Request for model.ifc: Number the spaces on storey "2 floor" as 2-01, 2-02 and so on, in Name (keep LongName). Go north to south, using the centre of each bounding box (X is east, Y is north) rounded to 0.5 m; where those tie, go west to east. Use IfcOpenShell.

First a look at what the model holds.

```python
import ifcopenshell
import ifcopenshell.util.element
import ifcopenshell.util.placement

model = ifcopenshell.open("model.ifc")
print(model.schema)
storey = next(s for s in model.by_type("IfcBuildingStorey") if s.Name == "2 floor")
spaces = [e for e in ifcopenshell.util.element.get_decomposition(storey) if e.is_a("IfcSpace")]
for e in sorted(spaces, key=lambda e: e.id()):
    origin = ifcopenshell.util.placement.get_local_placement(e.ObjectPlacement)[:3, 3]
    print(e.id(), e.Name, e.LongName, origin.round(2) + 0.0, sep=" | ")
```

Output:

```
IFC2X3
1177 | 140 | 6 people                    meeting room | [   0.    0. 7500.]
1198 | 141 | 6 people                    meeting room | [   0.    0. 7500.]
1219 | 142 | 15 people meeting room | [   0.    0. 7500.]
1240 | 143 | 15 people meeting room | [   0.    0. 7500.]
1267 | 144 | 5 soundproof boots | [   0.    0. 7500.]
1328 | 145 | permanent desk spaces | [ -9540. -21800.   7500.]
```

```python
import ifcopenshell
import ifcopenshell.geom
import ifcopenshell.util.element
import ifcopenshell.util.shape

model = ifcopenshell.open("model.ifc")
settings = ifcopenshell.geom.settings()
settings.set("use-world-coords", True)


def centre(element):
    shape = ifcopenshell.geom.create_shape(settings, element)
    return ifcopenshell.util.shape.get_bbox_centroid(shape.geometry)


storey = next(s for s in model.by_type("IfcBuildingStorey") if s.Name == "2 floor")
spaces = [e for e in ifcopenshell.util.element.get_decomposition(storey) if e.is_a("IfcSpace")]

# Insertion points can sit at a corner or the storey origin, so sort by the geometry (in metres).
centres = {e: centre(e) for e in spaces}
spaces.sort(key=lambda e: (-round(centres[e][1] / 0.5), centres[e][0]))

for i, e in enumerate(spaces, start=1):
    number = f"2-{i:02d}"
    e.Name = number
    print(e.id(), number)

model.write("model_v2.ifc")
```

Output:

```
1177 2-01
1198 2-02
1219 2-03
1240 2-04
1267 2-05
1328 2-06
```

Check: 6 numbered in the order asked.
